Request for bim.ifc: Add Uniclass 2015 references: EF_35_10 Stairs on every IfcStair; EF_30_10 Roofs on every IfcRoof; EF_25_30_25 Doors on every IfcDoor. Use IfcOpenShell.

First a look at what the model holds.

```python
import ifcopenshell

model = ifcopenshell.open("bim.ifc")
print(model.schema)
print("classifications:", [c.Name for c in model.by_type("IfcClassification")])
for ifc_class in ("IfcDoor", "IfcRoof", "IfcStair", "IfcWall", "IfcWindow"):
    print(ifc_class, len(model.by_type(ifc_class)))
```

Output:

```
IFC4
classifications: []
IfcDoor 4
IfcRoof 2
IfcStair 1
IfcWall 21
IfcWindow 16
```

```python
import ifcopenshell
import ifcopenshell.api.classification

model = ifcopenshell.open("bim.ifc")

system = ifcopenshell.api.classification.add_classification(model, classification="Uniclass 2015")

codes = {
    "IfcStair": ("EF_35_10", "Stairs"),
    "IfcRoof": ("EF_30_10", "Roofs"),
    "IfcDoor": ("EF_25_30_25", "Doors"),
}
for ifc_class, (code, name) in codes.items():
    products = model.by_type(ifc_class)
    ifcopenshell.api.classification.add_reference(
        model, products=products, classification=system, identification=code, name=name
    )
    print(code, len(products))

model.write("bim_v2.ifc")
```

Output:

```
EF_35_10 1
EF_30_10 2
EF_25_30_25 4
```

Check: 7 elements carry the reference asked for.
